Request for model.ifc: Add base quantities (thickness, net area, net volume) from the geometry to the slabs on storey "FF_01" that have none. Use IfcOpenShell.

First a look at what the model holds.

```python
import ifcopenshell
import ifcopenshell.util.element
import ifcopenshell.util.unit

model = ifcopenshell.open("model.ifc")
print(model.schema)
for unit_type in ("LENGTHUNIT", "AREAUNIT", "VOLUMEUNIT"):
    print(unit_type, ifcopenshell.util.unit.calculate_unit_scale(model, unit_type))
storey = next(s for s in model.by_type("IfcBuildingStorey") if s.Name == "FF_01")
slabs = [e for e in ifcopenshell.util.element.get_decomposition(storey) if e.is_a("IfcSlab")]
for e in sorted(slabs, key=lambda e: e.id()):
    print(e.id(), e.is_a(), e.Name, list(ifcopenshell.util.element.get_psets(e, qtos_only=True)), sep=" | ")
```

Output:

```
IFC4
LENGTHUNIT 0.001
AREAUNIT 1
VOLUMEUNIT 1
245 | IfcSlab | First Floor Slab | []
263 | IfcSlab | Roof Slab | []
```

```python
import ifcopenshell
import ifcopenshell.api.pset
import ifcopenshell.geom
import ifcopenshell.util.element
import ifcopenshell.util.shape
import ifcopenshell.util.unit

model = ifcopenshell.open("model.ifc")
unit_scale = ifcopenshell.util.unit.calculate_unit_scale(model)
area_scale = ifcopenshell.util.unit.calculate_unit_scale(model, "AREAUNIT")
volume_scale = ifcopenshell.util.unit.calculate_unit_scale(model, "VOLUMEUNIT")
settings = ifcopenshell.geom.settings()

storey = next(s for s in model.by_type("IfcBuildingStorey") if s.Name == "FF_01")
slabs = [e for e in ifcopenshell.util.element.get_decomposition(storey) if e.is_a("IfcSlab")]

for e in sorted(slabs, key=lambda e: e.id()):
    if ifcopenshell.util.element.get_psets(e, qtos_only=True, should_inherit=False):
        continue
    # Geometry comes back in metres, in the element's own axes.
    shape = ifcopenshell.geom.create_shape(settings, e)
    values = {
        "Width": ifcopenshell.util.shape.get_z(shape.geometry) / unit_scale,
        "NetArea": ifcopenshell.util.shape.get_footprint_area(shape.geometry) / area_scale,
        "NetVolume": ifcopenshell.util.shape.get_volume(shape.geometry) / volume_scale,
    }
    qto = ifcopenshell.api.pset.add_qto(model, product=e, name="Qto_SlabBaseQuantities")
    ifcopenshell.api.pset.edit_qto(model, qto=qto, properties=values)
    print(e.id(), {k: round(v, 3) for k, v in values.items()})

model.write("model_edited.ifc")
```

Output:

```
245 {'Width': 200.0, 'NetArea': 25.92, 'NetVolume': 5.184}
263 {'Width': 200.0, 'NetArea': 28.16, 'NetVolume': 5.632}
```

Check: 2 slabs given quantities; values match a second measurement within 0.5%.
